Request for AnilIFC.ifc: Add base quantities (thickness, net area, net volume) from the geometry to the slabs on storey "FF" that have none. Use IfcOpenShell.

First a look at what the model holds.

```python
import ifcopenshell
import ifcopenshell.util.element
import ifcopenshell.util.unit

model = ifcopenshell.open("AnilIFC.ifc")
print(model.schema)
for unit_type in ("LENGTHUNIT", "AREAUNIT", "VOLUMEUNIT"):
    print(unit_type, ifcopenshell.util.unit.calculate_unit_scale(model, unit_type))
storey = next(s for s in model.by_type("IfcBuildingStorey") if s.Name == "FF")
slabs = [e for e in ifcopenshell.util.element.get_decomposition(storey) if e.is_a("IfcSlab")]
for e in sorted(slabs, key=lambda e: e.id()):
    print(e.id(), e.is_a(), e.Name, list(ifcopenshell.util.element.get_psets(e, qtos_only=True)), sep=" | ")
```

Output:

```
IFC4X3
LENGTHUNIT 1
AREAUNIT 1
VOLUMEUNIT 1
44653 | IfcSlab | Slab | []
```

```python
import ifcopenshell
import ifcopenshell.api.pset
import ifcopenshell.geom
import ifcopenshell.util.element
import ifcopenshell.util.shape
import ifcopenshell.util.unit

model = ifcopenshell.open("AnilIFC.ifc")
unit_scale = ifcopenshell.util.unit.calculate_unit_scale(model)
area_scale = ifcopenshell.util.unit.calculate_unit_scale(model, "AREAUNIT")
volume_scale = ifcopenshell.util.unit.calculate_unit_scale(model, "VOLUMEUNIT")
settings = ifcopenshell.geom.settings()

storey = next(s for s in model.by_type("IfcBuildingStorey") if s.Name == "FF")
slabs = [e for e in ifcopenshell.util.element.get_decomposition(storey) if e.is_a("IfcSlab")]

for e in sorted(slabs, key=lambda e: e.id()):
    if ifcopenshell.util.element.get_psets(e, qtos_only=True, should_inherit=False):
        continue
    # Geometry comes back in metres, in the element's own axes.
    shape = ifcopenshell.geom.create_shape(settings, e)
    values = {
        "Width": ifcopenshell.util.shape.get_z(shape.geometry) / unit_scale,
        "NetArea": ifcopenshell.util.shape.get_footprint_area(shape.geometry) / area_scale,
        "NetVolume": ifcopenshell.util.shape.get_volume(shape.geometry) / volume_scale,
    }
    qto = ifcopenshell.api.pset.add_qto(model, product=e, name="Qto_SlabBaseQuantities")
    ifcopenshell.api.pset.edit_qto(model, qto=qto, properties=values)
    print(e.id(), {k: round(v, 3) for k, v in values.items()})

model.write("AnilIFC_v2.ifc")
```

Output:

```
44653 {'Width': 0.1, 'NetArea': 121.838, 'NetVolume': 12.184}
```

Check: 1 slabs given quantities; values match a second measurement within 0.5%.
